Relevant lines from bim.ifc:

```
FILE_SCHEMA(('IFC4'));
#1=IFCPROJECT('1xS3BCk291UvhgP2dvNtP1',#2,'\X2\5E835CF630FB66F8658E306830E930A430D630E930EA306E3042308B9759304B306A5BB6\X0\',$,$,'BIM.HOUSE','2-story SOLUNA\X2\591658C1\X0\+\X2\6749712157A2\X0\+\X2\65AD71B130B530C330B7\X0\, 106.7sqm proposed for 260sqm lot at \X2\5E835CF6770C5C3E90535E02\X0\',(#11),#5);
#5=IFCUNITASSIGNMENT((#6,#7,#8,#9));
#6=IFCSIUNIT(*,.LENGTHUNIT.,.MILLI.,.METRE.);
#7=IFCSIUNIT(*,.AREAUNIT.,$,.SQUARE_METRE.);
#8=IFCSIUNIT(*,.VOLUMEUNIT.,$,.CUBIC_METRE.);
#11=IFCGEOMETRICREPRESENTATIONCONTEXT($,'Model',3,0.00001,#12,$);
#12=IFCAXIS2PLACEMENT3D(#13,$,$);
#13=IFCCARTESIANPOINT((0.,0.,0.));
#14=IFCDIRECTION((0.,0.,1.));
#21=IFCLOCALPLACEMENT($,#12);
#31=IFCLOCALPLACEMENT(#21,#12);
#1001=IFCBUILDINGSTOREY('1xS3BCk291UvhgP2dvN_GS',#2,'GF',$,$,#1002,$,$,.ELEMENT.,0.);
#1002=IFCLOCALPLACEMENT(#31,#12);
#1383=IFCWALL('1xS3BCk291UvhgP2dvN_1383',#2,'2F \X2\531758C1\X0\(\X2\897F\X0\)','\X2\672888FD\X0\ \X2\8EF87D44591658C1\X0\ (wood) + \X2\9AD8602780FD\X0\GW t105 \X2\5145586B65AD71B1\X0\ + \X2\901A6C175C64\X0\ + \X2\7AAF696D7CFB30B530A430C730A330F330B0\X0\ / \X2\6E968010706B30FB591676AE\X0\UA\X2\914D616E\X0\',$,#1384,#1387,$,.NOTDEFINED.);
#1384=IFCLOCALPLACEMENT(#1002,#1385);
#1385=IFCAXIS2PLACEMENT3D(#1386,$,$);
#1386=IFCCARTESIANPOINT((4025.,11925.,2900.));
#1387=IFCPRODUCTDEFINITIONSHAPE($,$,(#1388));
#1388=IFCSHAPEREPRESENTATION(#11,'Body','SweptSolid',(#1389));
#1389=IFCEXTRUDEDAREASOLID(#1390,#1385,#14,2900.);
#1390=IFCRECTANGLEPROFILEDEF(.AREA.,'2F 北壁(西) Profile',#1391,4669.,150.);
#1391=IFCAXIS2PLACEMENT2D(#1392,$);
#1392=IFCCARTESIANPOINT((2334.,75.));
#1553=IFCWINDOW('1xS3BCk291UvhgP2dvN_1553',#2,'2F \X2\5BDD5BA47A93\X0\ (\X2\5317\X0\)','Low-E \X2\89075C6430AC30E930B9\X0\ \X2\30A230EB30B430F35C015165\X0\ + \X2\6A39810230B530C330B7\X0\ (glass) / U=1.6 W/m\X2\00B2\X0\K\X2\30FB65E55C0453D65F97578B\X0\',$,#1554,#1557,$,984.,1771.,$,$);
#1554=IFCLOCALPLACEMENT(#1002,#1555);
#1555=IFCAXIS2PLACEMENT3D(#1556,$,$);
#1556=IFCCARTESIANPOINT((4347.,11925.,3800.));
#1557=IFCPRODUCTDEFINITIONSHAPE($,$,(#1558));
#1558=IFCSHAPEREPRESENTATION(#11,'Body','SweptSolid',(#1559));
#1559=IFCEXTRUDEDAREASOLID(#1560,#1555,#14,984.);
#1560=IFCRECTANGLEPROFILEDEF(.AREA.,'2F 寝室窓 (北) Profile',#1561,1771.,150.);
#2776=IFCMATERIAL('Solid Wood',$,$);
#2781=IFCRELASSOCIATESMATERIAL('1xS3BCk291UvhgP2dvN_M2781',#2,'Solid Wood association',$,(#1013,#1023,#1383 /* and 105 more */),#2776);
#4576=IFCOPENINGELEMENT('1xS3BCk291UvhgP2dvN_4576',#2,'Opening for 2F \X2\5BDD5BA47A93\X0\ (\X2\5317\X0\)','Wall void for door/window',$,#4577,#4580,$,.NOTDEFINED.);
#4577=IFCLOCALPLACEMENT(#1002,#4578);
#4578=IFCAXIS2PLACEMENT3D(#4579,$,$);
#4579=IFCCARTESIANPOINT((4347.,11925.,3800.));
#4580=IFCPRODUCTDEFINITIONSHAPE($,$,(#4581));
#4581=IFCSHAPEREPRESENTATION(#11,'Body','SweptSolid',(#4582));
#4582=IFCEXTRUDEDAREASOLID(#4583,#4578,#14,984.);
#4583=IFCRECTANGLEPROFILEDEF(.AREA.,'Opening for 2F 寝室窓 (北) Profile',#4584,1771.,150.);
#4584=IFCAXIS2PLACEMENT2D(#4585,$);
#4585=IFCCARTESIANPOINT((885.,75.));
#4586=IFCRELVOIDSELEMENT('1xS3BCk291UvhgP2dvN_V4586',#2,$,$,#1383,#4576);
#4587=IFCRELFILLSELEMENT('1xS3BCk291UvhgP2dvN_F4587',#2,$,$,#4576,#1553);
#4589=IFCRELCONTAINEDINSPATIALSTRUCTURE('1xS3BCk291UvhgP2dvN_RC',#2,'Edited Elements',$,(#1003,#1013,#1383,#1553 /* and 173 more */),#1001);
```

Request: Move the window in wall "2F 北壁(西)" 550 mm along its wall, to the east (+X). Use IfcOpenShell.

```python
import ifcopenshell
import ifcopenshell.api.geometry
import ifcopenshell.util.placement

model = ifcopenshell.open("bim.ifc")

window = model.by_guid("1xS3BCk291UvhgP2dvN_1553")
opening = window.FillsVoids[0].RelatingOpeningElement
wall = opening.VoidsElements[0].RelatingBuildingElement

wall_matrix = ifcopenshell.util.placement.get_local_placement(wall.ObjectPlacement)
shift = wall_matrix[:3, 0] * 550.0
before = ifcopenshell.util.placement.get_local_placement(window.ObjectPlacement)[:3, 3].copy()

# The window is not placed relative to its opening, so move both.
for product in (opening, window):
    matrix = ifcopenshell.util.placement.get_local_placement(product.ObjectPlacement)
    matrix[:3, 3] += shift
    ifcopenshell.api.geometry.edit_object_placement(model, product=product, matrix=matrix, is_si=False)

after = ifcopenshell.util.placement.get_local_placement(window.ObjectPlacement)[:3, 3]
print("window moved by", (after - before).round(3) + 0.0)

model.write("bim_rev.ifc")
```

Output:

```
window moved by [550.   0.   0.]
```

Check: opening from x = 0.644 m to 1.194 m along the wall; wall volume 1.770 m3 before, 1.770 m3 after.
